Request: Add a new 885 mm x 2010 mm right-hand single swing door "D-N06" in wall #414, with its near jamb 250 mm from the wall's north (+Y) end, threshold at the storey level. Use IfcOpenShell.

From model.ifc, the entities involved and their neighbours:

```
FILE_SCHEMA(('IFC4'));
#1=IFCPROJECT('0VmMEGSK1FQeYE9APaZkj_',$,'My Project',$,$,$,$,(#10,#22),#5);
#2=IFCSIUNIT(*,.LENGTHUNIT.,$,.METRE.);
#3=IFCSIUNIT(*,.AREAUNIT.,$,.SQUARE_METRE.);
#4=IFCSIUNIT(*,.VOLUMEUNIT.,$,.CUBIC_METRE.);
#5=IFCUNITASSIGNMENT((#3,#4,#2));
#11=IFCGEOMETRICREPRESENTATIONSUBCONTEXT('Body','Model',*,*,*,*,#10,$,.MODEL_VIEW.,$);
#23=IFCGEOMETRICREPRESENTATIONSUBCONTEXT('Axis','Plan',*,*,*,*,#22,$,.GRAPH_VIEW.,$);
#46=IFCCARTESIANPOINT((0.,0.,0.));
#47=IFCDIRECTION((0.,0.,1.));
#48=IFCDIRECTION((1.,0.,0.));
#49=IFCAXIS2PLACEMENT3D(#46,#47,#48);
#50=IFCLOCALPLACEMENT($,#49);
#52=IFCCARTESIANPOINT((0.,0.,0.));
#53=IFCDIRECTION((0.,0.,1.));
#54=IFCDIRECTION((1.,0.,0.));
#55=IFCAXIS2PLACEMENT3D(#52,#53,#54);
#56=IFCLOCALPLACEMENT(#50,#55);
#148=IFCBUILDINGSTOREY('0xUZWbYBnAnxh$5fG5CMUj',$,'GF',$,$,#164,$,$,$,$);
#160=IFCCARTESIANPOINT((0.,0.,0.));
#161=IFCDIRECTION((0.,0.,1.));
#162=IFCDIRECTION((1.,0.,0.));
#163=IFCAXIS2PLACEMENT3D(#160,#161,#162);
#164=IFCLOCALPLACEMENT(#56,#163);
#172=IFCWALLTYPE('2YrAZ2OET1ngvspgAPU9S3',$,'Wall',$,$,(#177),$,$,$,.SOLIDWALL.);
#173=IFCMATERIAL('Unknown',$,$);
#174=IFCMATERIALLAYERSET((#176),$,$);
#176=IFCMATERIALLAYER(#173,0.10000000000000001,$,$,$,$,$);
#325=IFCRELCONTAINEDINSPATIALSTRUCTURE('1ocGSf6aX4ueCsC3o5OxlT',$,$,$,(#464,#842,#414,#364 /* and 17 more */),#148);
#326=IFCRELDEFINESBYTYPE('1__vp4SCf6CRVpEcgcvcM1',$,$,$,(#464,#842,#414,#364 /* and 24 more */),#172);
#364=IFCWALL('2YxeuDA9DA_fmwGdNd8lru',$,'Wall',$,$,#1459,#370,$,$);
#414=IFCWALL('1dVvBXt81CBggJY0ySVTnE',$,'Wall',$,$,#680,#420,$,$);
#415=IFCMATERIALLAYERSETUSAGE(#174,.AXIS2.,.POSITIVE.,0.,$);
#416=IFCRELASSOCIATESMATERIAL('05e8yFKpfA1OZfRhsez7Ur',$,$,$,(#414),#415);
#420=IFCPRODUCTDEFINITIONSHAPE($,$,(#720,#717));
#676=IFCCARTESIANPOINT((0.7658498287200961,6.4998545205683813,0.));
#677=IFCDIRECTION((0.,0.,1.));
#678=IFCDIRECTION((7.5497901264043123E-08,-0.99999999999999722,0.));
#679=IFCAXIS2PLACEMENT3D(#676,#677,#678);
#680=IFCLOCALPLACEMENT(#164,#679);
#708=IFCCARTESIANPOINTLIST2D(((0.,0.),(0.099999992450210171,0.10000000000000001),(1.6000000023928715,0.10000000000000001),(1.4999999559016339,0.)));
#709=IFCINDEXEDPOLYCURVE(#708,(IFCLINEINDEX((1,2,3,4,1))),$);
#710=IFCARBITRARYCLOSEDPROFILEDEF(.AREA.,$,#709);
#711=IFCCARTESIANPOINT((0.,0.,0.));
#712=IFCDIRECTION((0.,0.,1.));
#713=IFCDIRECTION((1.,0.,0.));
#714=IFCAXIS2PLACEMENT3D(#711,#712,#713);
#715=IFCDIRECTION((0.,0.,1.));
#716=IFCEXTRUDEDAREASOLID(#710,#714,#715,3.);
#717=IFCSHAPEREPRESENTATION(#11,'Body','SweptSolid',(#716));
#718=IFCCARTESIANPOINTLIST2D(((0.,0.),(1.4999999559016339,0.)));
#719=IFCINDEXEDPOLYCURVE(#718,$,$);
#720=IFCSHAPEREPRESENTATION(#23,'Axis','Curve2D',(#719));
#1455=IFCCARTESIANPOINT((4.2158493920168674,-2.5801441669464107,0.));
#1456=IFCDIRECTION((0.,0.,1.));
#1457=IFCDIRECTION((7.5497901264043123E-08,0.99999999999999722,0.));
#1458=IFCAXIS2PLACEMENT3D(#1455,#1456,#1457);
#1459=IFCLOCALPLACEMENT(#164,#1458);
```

```python
import numpy as np
import ifcopenshell
import ifcopenshell.api.feature
import ifcopenshell.api.geometry
import ifcopenshell.api.root
import ifcopenshell.api.spatial
import ifcopenshell.geom
import ifcopenshell.util.element
import ifcopenshell.util.placement
import ifcopenshell.util.representation
import ifcopenshell.util.shape
import ifcopenshell.util.unit

model = ifcopenshell.open("model.ifc")
unit_scale = ifcopenshell.util.unit.calculate_unit_scale(model)
settings = ifcopenshell.geom.settings()


def volume(element):
    """Net volume in cubic metres, openings subtracted."""
    shape = ifcopenshell.geom.create_shape(settings, element)
    return ifcopenshell.util.shape.get_volume(shape.geometry)


wall = model.by_guid("1dVvBXt81CBggJY0ySVTnE")
storey = ifcopenshell.util.element.get_container(wall, ifc_class="IfcBuildingStorey")
context = ifcopenshell.util.representation.get_context(model, "Model", "Body", "MODEL_VIEW")
before = volume(wall)

width, height, from_end, sill = 0.885, 2.01, 0.25, 0.0  # metres

# The wall runs along its own X axis, and the end named is its -X end.
wall_shape = ifcopenshell.geom.create_shape(settings, wall)
x, y, z = ifcopenshell.util.shape.get_vertices(wall_shape.geometry).T
start = x.min() + from_end
face, thickness = float(y.min()), float(y.max() - y.min())
wall_matrix = ifcopenshell.util.placement.get_local_placement(wall.ObjectPlacement)
level = ifcopenshell.util.placement.get_local_placement(storey.ObjectPlacement)[2, 3]


def in_wall(x, y):
    """Placement at x, y metres in the wall's axes, at sill height."""
    matrix = wall_matrix.copy()
    matrix[:, 3] = wall_matrix @ np.array([x / unit_scale, y / unit_scale, 0.0, 1.0])
    matrix[2, 3] = level + sill / unit_scale
    return matrix


# Opening: a box that overshoots both wall faces by 50 mm.
opening = ifcopenshell.api.root.create_entity(model, ifc_class="IfcOpeningElement", predefined_type="OPENING")
box = ifcopenshell.api.geometry.add_wall_representation(
    model, context=context, length=width, height=height, thickness=thickness + 0.1
)
ifcopenshell.api.geometry.assign_representation(model, product=opening, representation=box)
ifcopenshell.api.geometry.edit_object_placement(model, product=opening, matrix=in_wall(start, face - 0.05), is_si=False)
ifcopenshell.api.feature.add_feature(model, feature=opening, element=wall)

door = ifcopenshell.api.root.create_entity(model, ifc_class="IfcDoor", name="D-N06", predefined_type="DOOR")
door.OverallWidth, door.OverallHeight = width / unit_scale, height / unit_scale
door.OperationType = "SINGLE_SWING_RIGHT"
body = ifcopenshell.api.geometry.add_door_representation(
    model,
    context=context,
    overall_width=door.OverallWidth,
    overall_height=door.OverallHeight,
    operation_type="SINGLE_SWING_RIGHT",
    lining_properties={"LiningDepth": thickness / unit_scale, "ThresholdDepth": thickness / unit_scale},
)
ifcopenshell.api.geometry.assign_representation(model, product=door, representation=body)
ifcopenshell.api.spatial.assign_container(model, products=[door], relating_structure=storey)
ifcopenshell.api.feature.add_filling(model, opening=opening, element=door)

# The lining spans the wall, so the door starts at the wall face.
ifcopenshell.api.geometry.edit_object_placement(model, product=door, matrix=in_wall(start, face), is_si=False)

after = volume(wall)

print(f"wall volume {before:.3f} -> {after:.3f} m3")

model.write("model-out.ifc")
```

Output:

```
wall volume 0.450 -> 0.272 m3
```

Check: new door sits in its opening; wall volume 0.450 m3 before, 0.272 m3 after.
